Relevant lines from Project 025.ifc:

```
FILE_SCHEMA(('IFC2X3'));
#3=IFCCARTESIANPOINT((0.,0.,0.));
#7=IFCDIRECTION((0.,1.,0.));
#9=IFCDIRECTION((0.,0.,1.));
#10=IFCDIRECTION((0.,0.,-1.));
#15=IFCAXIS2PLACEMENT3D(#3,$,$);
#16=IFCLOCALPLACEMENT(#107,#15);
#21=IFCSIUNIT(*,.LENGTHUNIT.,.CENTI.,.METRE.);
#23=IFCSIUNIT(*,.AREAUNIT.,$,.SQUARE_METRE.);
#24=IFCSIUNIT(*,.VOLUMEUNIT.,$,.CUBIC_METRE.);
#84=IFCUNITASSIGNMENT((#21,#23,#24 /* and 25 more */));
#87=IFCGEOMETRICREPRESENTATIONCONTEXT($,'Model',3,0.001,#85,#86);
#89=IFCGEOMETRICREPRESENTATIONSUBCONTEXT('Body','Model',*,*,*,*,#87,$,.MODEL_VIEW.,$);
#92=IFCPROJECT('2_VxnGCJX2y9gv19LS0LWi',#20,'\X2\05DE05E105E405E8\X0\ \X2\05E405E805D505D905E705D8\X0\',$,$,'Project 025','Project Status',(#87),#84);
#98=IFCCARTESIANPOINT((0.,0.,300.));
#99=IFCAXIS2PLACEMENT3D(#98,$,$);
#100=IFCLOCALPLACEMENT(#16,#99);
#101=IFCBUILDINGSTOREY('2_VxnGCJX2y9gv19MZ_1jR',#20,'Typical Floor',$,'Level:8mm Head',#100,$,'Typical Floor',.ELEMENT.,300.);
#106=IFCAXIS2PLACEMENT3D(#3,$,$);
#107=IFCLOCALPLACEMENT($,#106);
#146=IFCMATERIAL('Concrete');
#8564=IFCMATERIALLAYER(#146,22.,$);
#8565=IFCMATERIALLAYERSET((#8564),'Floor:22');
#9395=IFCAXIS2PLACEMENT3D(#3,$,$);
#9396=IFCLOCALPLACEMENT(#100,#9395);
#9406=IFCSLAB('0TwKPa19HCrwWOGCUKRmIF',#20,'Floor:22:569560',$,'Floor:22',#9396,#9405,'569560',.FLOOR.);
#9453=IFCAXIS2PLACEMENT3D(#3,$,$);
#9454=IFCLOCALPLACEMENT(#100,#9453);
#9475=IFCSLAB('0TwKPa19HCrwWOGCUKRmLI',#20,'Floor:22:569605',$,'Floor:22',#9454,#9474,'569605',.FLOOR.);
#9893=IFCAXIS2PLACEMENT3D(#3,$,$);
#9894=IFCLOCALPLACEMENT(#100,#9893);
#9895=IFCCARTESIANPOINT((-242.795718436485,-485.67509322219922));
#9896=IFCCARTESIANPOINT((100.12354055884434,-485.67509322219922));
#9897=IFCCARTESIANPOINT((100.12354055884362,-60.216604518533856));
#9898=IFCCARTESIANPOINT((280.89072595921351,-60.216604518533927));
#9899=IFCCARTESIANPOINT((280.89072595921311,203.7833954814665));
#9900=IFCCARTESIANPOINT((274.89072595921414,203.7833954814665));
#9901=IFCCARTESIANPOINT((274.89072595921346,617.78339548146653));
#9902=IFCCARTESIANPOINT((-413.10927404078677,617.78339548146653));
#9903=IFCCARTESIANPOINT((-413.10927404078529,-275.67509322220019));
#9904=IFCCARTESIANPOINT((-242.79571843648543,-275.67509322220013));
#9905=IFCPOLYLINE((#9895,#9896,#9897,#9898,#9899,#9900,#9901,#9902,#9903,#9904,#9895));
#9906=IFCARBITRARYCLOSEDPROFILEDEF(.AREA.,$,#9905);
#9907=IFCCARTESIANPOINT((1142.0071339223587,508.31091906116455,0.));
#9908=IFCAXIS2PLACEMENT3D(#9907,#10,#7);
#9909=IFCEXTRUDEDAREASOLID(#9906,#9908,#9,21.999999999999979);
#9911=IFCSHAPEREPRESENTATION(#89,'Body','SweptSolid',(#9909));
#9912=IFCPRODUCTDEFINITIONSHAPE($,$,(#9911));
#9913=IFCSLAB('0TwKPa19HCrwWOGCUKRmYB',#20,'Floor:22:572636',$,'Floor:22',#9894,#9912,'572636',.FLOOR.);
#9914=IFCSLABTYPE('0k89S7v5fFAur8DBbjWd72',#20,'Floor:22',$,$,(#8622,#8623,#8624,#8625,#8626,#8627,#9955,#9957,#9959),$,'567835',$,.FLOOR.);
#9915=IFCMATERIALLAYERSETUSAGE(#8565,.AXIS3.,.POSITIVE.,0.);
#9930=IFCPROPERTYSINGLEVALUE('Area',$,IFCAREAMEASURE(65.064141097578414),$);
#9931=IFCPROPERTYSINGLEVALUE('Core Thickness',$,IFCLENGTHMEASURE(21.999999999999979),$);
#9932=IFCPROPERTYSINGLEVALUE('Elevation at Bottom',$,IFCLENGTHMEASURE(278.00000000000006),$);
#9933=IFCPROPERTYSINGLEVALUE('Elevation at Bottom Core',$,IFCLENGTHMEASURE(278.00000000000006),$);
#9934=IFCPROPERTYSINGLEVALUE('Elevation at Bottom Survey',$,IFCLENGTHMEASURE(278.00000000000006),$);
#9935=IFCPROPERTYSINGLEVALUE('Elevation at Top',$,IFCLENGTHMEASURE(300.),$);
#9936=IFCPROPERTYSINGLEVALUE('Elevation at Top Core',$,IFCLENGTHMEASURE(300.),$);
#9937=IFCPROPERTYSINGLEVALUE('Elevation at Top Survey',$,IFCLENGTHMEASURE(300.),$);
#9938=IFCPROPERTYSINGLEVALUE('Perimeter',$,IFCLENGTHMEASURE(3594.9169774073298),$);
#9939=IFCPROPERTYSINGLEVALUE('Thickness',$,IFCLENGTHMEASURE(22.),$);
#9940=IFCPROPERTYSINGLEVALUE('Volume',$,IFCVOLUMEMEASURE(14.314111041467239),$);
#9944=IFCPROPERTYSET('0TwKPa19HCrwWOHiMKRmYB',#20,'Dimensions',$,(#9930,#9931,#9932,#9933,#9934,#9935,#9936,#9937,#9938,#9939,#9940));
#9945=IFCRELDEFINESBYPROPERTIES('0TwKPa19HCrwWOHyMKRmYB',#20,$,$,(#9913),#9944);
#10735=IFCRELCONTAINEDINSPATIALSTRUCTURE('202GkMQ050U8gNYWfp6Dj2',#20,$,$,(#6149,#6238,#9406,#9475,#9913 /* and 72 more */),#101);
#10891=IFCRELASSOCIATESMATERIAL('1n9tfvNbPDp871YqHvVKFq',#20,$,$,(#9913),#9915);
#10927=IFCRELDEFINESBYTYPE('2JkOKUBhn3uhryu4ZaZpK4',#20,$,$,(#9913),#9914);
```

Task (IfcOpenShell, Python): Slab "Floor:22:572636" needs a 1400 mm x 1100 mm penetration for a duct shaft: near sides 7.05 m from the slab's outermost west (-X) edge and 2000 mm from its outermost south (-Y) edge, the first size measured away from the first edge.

```python
import numpy as np
import ifcopenshell
import ifcopenshell.api.feature
import ifcopenshell.api.geometry
import ifcopenshell.api.pset
import ifcopenshell.api.root
import ifcopenshell.geom
import ifcopenshell.util.element
import ifcopenshell.util.placement
import ifcopenshell.util.representation
import ifcopenshell.util.shape
import ifcopenshell.util.unit

model = ifcopenshell.open("Project 025.ifc")
unit_scale = ifcopenshell.util.unit.calculate_unit_scale(model)
area_scale = ifcopenshell.util.unit.calculate_unit_scale(model, "AREAUNIT")
volume_scale = ifcopenshell.util.unit.calculate_unit_scale(model, "VOLUMEUNIT")
settings = ifcopenshell.geom.settings()


def volume(element):
    """Net volume in cubic metres, openings subtracted."""
    shape = ifcopenshell.geom.create_shape(settings, element)
    return ifcopenshell.util.shape.get_volume(shape.geometry)


slab = model.by_guid("0TwKPa19HCrwWOGCUKRmYB")
before = volume(slab)

# Extent in the slab's own axes, in metres. The edges named are its -X and -Y sides.
slab_shape = ifcopenshell.geom.create_shape(settings, slab)
vertices = ifcopenshell.util.shape.get_vertices(slab_shape.geometry)
x_min, y_min, bottom = vertices.min(axis=0)
top = vertices[:, 2].max()

opening = ifcopenshell.api.root.create_entity(model, ifc_class="IfcOpeningElement", name="Duct shaft opening")
context = ifcopenshell.util.representation.get_context(model, "Model", "Body", "MODEL_VIEW")
width, depth = 1.4, 1.1
outline = [(0.0, 0.0), (width, 0.0), (width, depth), (0.0, depth), (0.0, 0.0)]
# Overshoot both faces by 50 mm so the cut is clean.
shape = ifcopenshell.api.geometry.add_slab_representation(
    model, context=context, depth=top - bottom + 0.1, polyline=outline
)
ifcopenshell.api.geometry.assign_representation(model, product=opening, representation=shape)

matrix = ifcopenshell.util.placement.get_local_placement(slab.ObjectPlacement)
matrix[:, 3] = matrix @ np.append(np.array([x_min + 7.05, y_min + 2, bottom - 0.05]) / unit_scale, 1.0)
ifcopenshell.api.geometry.edit_object_placement(model, product=opening, matrix=matrix, is_si=False)
ifcopenshell.api.feature.add_feature(model, feature=opening, element=slab)

after = volume(slab)

# Update the slab's stored quantities.
pset = model.by_id(ifcopenshell.util.element.get_pset(slab, "Dimensions", should_inherit=False)["id"])
ifcopenshell.api.pset.edit_pset(model, pset=pset, properties={
    "Area": model.create_entity("IfcAreaMeasure", after / (top - bottom) / area_scale),
    "Volume": model.create_entity("IfcVolumeMeasure", after / volume_scale),
})

print(f"slab volume {before:.3f} -> {after:.3f} m3")

model.write("Project 025_updated.ifc")
```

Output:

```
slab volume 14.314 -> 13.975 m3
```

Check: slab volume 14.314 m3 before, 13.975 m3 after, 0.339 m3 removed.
